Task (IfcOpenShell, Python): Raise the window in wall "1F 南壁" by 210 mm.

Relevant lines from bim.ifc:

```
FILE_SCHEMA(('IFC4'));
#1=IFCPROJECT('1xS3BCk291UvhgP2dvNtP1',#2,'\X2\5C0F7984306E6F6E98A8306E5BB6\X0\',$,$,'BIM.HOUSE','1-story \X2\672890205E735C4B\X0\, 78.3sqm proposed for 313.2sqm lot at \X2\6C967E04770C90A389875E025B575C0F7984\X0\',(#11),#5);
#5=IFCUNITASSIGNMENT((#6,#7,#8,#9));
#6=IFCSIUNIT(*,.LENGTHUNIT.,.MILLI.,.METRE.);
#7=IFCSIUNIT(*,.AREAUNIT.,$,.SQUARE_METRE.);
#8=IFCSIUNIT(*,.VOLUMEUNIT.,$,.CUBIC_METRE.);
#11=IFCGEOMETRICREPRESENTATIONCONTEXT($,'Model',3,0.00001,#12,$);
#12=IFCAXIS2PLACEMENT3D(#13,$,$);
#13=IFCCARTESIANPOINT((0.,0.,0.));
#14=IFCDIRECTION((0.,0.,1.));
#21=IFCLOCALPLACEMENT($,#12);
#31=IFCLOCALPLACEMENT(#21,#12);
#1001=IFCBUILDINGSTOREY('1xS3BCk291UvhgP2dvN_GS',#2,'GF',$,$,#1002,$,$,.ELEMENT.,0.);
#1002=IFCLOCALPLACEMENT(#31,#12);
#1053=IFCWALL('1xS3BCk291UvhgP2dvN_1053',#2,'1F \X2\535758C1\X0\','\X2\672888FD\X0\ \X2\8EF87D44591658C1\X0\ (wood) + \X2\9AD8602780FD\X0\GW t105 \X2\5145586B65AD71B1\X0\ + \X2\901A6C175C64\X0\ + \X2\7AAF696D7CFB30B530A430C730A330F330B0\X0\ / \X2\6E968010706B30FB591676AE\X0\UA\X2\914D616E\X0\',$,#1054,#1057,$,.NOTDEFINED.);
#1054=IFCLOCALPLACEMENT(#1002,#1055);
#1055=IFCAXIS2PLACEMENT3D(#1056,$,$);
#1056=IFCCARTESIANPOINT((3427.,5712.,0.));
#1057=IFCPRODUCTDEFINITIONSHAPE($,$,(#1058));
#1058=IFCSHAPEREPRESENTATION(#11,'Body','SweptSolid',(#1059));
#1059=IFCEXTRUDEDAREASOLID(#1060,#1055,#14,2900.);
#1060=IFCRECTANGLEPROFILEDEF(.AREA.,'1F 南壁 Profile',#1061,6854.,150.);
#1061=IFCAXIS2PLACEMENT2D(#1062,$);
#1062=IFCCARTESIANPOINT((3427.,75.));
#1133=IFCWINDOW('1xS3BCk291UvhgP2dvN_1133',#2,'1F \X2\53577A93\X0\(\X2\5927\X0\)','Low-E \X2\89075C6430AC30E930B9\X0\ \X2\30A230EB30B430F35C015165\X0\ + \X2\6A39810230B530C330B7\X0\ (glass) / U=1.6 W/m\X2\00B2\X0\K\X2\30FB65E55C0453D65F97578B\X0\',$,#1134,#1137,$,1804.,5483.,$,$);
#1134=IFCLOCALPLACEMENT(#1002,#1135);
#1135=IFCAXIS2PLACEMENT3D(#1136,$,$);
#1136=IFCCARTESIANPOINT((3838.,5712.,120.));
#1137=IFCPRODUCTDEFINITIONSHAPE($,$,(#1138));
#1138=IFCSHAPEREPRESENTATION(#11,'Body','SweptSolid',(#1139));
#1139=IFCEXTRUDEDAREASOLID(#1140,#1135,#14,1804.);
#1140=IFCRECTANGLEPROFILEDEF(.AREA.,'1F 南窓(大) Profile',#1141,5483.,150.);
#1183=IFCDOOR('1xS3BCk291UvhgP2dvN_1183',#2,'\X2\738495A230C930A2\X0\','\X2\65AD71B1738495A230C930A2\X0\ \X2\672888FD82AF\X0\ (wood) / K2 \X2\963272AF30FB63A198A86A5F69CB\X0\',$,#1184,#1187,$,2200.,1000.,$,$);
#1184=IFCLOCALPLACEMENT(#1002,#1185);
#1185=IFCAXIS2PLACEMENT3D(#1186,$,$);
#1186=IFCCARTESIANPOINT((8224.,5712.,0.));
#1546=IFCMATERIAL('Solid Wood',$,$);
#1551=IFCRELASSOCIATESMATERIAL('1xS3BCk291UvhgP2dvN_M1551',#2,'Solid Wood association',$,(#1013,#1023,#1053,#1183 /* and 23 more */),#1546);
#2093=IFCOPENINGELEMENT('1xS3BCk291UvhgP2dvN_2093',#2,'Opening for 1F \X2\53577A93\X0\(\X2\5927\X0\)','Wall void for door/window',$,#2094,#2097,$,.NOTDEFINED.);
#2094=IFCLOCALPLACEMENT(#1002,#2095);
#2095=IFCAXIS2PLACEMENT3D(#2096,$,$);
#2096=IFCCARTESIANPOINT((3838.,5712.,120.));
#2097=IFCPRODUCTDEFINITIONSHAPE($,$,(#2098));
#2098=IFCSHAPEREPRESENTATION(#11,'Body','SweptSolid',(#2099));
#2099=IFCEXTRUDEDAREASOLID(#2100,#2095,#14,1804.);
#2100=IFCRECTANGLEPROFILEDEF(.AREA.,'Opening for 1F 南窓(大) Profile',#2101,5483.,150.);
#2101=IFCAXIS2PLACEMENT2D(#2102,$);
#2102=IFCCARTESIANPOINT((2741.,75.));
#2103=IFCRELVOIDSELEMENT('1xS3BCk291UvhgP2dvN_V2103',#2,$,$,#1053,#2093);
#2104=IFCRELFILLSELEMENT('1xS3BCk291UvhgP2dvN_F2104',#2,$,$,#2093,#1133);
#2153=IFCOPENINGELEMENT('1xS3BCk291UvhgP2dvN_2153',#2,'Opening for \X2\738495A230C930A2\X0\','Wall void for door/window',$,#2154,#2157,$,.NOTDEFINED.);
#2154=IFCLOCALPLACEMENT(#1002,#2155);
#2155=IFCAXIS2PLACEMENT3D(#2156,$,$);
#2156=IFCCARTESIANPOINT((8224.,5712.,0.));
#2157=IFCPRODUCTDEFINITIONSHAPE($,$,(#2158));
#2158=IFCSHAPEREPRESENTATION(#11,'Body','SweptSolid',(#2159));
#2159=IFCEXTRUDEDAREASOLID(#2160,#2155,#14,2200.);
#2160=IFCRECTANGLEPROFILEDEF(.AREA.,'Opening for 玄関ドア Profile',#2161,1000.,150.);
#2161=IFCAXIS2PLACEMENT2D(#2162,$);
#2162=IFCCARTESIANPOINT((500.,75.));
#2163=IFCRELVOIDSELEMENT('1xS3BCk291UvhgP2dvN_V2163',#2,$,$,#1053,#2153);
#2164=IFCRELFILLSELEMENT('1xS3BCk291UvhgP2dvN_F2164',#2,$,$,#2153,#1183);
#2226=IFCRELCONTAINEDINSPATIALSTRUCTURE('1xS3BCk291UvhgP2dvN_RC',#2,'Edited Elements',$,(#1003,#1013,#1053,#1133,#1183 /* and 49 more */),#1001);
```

```python
import numpy as np
import ifcopenshell
import ifcopenshell.api.geometry
import ifcopenshell.util.placement
import ifcopenshell.util.unit

model = ifcopenshell.open("bim.ifc")
unit_scale = ifcopenshell.util.unit.calculate_unit_scale(model)

window = model.by_guid("1xS3BCk291UvhgP2dvN_1133")
opening = window.FillsVoids[0].RelatingOpeningElement
dz = 0.21 / unit_scale

shift = np.array([0.0, 0.0, dz])
# The window is not placed relative to its opening, so move both.
for product in (opening, window):
    matrix = ifcopenshell.util.placement.get_local_placement(product.ObjectPlacement)
    matrix[:3, 3] += shift
    ifcopenshell.api.geometry.edit_object_placement(model, product=product, matrix=matrix, is_si=False)

print(f"moved by {dz * unit_scale:+.3f} m")

model.write("bim_v2.ifc")
```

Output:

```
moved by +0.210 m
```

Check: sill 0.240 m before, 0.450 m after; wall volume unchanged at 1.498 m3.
